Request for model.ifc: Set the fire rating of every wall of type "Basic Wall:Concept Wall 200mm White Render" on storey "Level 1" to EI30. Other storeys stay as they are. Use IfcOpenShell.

First a look at what the model holds.

```python
import ifcopenshell
import ifcopenshell.util.element

model = ifcopenshell.open("model.ifc")
print(model.schema)
storey = next(s for s in model.by_type("IfcBuildingStorey") if s.Name == "Level 1")
walls = [e for e in ifcopenshell.util.element.get_decomposition(storey) if e.is_a("IfcWall")]
seen = {}
for e in walls:
    element_type = ifcopenshell.util.element.get_type(e)
    key = (element_type.Name if element_type != e and element_type else None, ifcopenshell.util.element.get_pset(e, "Pset_WallCommon", "FireRating"))
    seen[key] = seen.get(key, 0) + 1
for (name, value), count in sorted(seen.items(), key=str):
    print(count, "x", name, "|", value)
```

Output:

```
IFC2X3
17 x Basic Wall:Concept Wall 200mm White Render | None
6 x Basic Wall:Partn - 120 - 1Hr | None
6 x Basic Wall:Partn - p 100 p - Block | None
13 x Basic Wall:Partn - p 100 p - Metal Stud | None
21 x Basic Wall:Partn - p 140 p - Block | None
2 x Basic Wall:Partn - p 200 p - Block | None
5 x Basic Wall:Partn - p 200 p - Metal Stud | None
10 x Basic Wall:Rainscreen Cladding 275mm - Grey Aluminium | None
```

```python
import ifcopenshell
import ifcopenshell.api.pset
import ifcopenshell.util.element

model = ifcopenshell.open("model.ifc")

storey = next(s for s in model.by_type("IfcBuildingStorey") if s.Name == "Level 1")
walls = [e for e in ifcopenshell.util.element.get_decomposition(storey) if e.is_a("IfcWall")]

count = 0
for e in walls:
    element_type = ifcopenshell.util.element.get_type(e)
    if element_type in (None, e) or element_type.Name != "Basic Wall:Concept Wall 200mm White Render":
        continue
    found = ifcopenshell.util.element.get_pset(e, "Pset_WallCommon", should_inherit=False)
    if found:
        pset = model.by_id(found["id"])
        if len(ifcopenshell.util.element.get_elements_by_pset(pset)) > 1:
            pset = ifcopenshell.api.pset.unshare_pset(model, products=[e], pset=pset)[0]
    else:
        pset = ifcopenshell.api.pset.add_pset(model, product=e, name="Pset_WallCommon")
    ifcopenshell.api.pset.edit_pset(model, pset=pset, properties={"FireRating": "EI30"})
    count += 1

print(count, "walls updated")

model.write("model_v2.ifc")
```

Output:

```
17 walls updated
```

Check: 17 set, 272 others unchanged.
